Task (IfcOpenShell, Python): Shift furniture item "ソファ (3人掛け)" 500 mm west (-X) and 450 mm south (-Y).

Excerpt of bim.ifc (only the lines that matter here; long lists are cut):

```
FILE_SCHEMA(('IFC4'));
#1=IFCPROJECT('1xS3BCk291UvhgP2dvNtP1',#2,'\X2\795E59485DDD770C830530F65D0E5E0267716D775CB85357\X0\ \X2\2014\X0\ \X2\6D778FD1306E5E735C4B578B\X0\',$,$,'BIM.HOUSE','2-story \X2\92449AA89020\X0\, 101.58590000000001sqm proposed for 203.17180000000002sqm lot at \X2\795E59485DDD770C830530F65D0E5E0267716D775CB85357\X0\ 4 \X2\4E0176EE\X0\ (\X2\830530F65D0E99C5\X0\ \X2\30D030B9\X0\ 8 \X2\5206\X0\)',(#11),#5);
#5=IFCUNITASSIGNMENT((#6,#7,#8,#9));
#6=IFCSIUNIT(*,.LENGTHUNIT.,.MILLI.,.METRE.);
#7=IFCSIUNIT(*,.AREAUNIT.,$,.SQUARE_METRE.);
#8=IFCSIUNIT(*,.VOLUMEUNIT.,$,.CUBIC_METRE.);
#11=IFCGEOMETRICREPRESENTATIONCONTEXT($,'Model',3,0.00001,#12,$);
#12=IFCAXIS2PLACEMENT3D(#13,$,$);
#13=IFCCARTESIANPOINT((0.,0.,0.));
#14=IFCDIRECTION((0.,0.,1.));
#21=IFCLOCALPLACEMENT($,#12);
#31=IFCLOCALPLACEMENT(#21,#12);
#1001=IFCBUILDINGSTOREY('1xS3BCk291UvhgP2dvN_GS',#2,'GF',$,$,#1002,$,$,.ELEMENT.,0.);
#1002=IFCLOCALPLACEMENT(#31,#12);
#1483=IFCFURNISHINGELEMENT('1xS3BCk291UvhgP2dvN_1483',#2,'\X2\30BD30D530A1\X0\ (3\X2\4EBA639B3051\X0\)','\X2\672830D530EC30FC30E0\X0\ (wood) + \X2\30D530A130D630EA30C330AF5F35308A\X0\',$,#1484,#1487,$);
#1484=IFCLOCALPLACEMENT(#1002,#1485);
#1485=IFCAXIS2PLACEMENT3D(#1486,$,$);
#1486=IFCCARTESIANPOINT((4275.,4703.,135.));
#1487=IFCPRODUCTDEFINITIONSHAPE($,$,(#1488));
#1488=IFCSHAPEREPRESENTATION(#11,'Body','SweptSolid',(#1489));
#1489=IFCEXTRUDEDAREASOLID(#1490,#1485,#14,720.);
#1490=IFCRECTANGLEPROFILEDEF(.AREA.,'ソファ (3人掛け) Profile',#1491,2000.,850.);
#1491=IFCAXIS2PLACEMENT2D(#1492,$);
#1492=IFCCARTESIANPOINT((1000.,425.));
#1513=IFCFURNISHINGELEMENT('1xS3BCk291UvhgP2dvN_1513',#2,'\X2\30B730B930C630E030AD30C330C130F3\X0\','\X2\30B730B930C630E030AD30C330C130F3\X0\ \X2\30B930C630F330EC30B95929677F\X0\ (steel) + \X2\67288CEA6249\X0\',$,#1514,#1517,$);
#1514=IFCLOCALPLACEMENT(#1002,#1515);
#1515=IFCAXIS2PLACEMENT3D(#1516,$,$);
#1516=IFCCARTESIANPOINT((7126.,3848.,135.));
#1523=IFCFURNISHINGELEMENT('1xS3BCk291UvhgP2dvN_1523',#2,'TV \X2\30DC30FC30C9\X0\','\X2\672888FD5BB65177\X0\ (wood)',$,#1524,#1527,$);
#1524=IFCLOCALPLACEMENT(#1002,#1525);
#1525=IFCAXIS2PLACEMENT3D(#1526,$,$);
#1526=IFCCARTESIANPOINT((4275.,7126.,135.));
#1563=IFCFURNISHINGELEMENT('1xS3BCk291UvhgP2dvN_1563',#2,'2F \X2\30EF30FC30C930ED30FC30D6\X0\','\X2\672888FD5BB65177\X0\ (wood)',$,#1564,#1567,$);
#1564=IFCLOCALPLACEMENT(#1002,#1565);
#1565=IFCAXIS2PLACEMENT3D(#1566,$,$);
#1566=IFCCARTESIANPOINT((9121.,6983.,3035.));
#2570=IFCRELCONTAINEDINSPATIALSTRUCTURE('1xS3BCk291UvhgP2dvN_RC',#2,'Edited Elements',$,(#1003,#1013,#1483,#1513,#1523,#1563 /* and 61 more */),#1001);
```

```python
import ifcopenshell
import ifcopenshell.api.geometry
import ifcopenshell.util.placement
import ifcopenshell.util.unit

model = ifcopenshell.open("bim.ifc")
unit_scale = ifcopenshell.util.unit.calculate_unit_scale(model)

item = model.by_guid("1xS3BCk291UvhgP2dvN_1483")
matrix = ifcopenshell.util.placement.get_local_placement(item.ObjectPlacement)
matrix[0, 3] -= 0.5 / unit_scale
matrix[1, 3] -= 0.45 / unit_scale
ifcopenshell.api.geometry.edit_object_placement(model, product=item, matrix=matrix, is_si=False)

print(ifcopenshell.util.placement.get_local_placement(item.ObjectPlacement).round(3) + 0.0)

model.write("bim_edited.ifc")
```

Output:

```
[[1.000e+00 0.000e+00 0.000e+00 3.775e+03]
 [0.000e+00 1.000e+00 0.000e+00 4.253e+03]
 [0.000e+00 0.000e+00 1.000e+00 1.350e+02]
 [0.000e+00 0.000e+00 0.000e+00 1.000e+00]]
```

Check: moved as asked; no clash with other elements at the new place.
